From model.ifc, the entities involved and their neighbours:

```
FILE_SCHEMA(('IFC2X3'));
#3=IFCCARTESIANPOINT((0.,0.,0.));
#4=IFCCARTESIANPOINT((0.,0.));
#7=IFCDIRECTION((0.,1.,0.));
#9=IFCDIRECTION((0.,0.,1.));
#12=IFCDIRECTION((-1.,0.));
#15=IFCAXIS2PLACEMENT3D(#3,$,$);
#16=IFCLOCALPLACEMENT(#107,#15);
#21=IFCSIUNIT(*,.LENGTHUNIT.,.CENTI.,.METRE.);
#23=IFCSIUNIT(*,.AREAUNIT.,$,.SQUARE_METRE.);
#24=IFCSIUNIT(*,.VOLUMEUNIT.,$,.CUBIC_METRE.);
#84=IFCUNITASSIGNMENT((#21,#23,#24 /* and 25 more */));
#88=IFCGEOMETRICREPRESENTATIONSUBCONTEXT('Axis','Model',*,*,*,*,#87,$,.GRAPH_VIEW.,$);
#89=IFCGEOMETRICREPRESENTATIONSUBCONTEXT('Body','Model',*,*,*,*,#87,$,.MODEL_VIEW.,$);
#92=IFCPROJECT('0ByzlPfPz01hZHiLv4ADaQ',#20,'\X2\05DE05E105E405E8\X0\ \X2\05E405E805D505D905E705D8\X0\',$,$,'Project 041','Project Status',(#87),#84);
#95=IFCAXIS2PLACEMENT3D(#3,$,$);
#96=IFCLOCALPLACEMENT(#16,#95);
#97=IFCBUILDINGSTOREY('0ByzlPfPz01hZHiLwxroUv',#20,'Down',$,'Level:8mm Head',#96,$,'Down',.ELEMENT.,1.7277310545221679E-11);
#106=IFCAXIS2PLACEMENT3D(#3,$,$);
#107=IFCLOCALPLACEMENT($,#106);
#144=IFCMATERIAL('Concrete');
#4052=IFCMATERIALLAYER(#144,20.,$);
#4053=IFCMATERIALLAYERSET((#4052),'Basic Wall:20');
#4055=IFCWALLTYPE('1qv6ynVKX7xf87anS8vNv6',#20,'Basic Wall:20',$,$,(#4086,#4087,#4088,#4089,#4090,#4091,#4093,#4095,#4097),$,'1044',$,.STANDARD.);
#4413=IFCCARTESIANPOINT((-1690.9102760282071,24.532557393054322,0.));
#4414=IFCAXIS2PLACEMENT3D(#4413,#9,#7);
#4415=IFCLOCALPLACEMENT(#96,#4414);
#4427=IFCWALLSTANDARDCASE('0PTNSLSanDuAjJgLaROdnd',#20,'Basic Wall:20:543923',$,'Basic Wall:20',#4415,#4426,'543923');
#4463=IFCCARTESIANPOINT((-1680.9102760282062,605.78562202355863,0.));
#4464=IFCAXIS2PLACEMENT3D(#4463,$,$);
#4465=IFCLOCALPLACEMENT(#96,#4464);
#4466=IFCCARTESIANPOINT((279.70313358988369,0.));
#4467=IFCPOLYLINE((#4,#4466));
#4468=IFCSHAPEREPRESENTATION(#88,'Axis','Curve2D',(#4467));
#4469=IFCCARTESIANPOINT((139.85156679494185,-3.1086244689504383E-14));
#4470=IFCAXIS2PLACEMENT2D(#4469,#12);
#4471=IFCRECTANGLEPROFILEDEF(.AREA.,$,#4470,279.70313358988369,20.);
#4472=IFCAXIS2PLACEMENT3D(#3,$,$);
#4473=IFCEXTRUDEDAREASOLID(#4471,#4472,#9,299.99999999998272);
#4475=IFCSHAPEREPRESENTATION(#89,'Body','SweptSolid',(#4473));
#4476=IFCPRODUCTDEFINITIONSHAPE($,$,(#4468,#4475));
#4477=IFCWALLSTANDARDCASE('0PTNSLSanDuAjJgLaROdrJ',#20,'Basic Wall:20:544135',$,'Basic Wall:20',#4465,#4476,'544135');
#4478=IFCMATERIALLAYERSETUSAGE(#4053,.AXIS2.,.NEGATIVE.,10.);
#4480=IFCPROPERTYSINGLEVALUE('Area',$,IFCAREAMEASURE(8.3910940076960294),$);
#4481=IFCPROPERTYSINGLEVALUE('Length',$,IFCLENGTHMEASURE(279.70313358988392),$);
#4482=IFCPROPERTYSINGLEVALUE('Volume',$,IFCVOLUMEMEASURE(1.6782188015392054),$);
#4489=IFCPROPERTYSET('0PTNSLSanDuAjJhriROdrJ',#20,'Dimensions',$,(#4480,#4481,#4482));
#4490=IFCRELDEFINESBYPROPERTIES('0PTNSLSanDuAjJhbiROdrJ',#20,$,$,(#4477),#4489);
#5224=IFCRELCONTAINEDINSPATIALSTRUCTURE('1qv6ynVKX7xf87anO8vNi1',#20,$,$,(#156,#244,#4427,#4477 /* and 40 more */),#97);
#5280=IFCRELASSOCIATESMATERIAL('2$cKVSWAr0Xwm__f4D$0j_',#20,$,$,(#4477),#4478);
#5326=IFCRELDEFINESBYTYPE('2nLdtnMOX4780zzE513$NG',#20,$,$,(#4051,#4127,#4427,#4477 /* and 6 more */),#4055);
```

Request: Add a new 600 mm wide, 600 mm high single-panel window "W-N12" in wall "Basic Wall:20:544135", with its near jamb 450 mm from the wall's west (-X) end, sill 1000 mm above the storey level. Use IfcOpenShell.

```python
import numpy as np
import ifcopenshell
import ifcopenshell.api.feature
import ifcopenshell.api.geometry
import ifcopenshell.api.pset
import ifcopenshell.api.root
import ifcopenshell.api.spatial
import ifcopenshell.api.type
import ifcopenshell.geom
import ifcopenshell.util.element
import ifcopenshell.util.placement
import ifcopenshell.util.representation
import ifcopenshell.util.shape
import ifcopenshell.util.unit

model = ifcopenshell.open("model.ifc")
unit_scale = ifcopenshell.util.unit.calculate_unit_scale(model)
area_scale = ifcopenshell.util.unit.calculate_unit_scale(model, "AREAUNIT")
volume_scale = ifcopenshell.util.unit.calculate_unit_scale(model, "VOLUMEUNIT")
settings = ifcopenshell.geom.settings()


def volume(element):
    """Net volume in cubic metres, openings subtracted."""
    shape = ifcopenshell.geom.create_shape(settings, element)
    return ifcopenshell.util.shape.get_volume(shape.geometry)


wall = model.by_guid("0PTNSLSanDuAjJgLaROdrJ")
storey = ifcopenshell.util.element.get_container(wall, ifc_class="IfcBuildingStorey")
context = ifcopenshell.util.representation.get_context(model, "Model", "Body", "MODEL_VIEW")
before = volume(wall)

width, height, from_end, sill = 0.6, 0.6, 0.45, 1  # metres

# The wall runs along its own X axis, and the end named is its -X end.
wall_shape = ifcopenshell.geom.create_shape(settings, wall)
x, y, z = ifcopenshell.util.shape.get_vertices(wall_shape.geometry).T
start = x.min() + from_end
face, thickness = float(y.min()), float(y.max() - y.min())
wall_matrix = ifcopenshell.util.placement.get_local_placement(wall.ObjectPlacement)
level = ifcopenshell.util.placement.get_local_placement(storey.ObjectPlacement)[2, 3]


def in_wall(x, y):
    """Placement at x, y metres in the wall's axes, at sill height."""
    matrix = wall_matrix.copy()
    matrix[:, 3] = wall_matrix @ np.array([x / unit_scale, y / unit_scale, 0.0, 1.0])
    matrix[2, 3] = level + sill / unit_scale
    return matrix


# Opening: a box that overshoots both wall faces by 50 mm.
opening = ifcopenshell.api.root.create_entity(model, ifc_class="IfcOpeningElement")
box = ifcopenshell.api.geometry.add_wall_representation(
    model, context=context, length=width, height=height, thickness=thickness + 0.1
)
ifcopenshell.api.geometry.assign_representation(model, product=opening, representation=box)
ifcopenshell.api.geometry.edit_object_placement(model, product=opening, matrix=in_wall(start, face - 0.05), is_si=False)
ifcopenshell.api.feature.add_feature(model, feature=opening, element=wall)

window = ifcopenshell.api.root.create_entity(model, ifc_class="IfcWindow", name="W-N12")
window.OverallWidth, window.OverallHeight = width / unit_scale, height / unit_scale
body = ifcopenshell.api.geometry.add_window_representation(
    model,
    context=context,
    overall_width=window.OverallWidth,
    overall_height=window.OverallHeight,
    partition_type="SINGLE_PANEL",
)
ifcopenshell.api.geometry.assign_representation(model, product=window, representation=body)
ifcopenshell.api.spatial.assign_container(model, products=[window], relating_structure=storey)
fills = ifcopenshell.api.feature.add_filling(model, opening=opening, element=window)
fills.OwnerHistory = window.OwnerHistory  # required in IFC2X3

# IFC2X3 keeps the operation on the window style.
style = ifcopenshell.api.root.create_entity(model, ifc_class="IfcWindowStyle", name="W-N12")
style.OperationType, style.ConstructionType = "SINGLE_PANEL", "NOTDEFINED"
style.ParameterTakesPrecedence = style.Sizeable = False
ifcopenshell.api.type.assign_type(model, related_objects=[window], relating_type=style)

# Centre the window in the wall's thickness.
ifcopenshell.api.geometry.edit_object_placement(model, product=window, matrix=in_wall(start, face), is_si=False)
window_shape = ifcopenshell.geom.create_shape(settings, window)
depth = ifcopenshell.util.shape.get_vertices(window_shape.geometry)[:, 1]
offset = face + thickness / 2 - (depth.min() + depth.max()) / 2
ifcopenshell.api.geometry.edit_object_placement(model, product=window, matrix=in_wall(start, offset), is_si=False)

after = volume(wall)

# Update the wall's stored quantities.
pset = model.by_id(ifcopenshell.util.element.get_pset(wall, "Dimensions", should_inherit=False)["id"])
ifcopenshell.api.pset.edit_pset(model, pset=pset, properties={
    "Area": model.create_entity("IfcAreaMeasure", after / thickness / area_scale),
    "Volume": model.create_entity("IfcVolumeMeasure", after / volume_scale),
})

print(f"wall volume {before:.3f} -> {after:.3f} m3")

model.write("model_v2.ifc")
```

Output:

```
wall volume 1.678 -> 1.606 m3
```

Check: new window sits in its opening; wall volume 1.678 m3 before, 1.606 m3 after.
